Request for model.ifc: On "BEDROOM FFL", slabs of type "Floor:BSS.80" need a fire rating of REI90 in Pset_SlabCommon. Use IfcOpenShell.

First a look at what the model holds.

```python
import ifcopenshell
import ifcopenshell.util.element

model = ifcopenshell.open("model.ifc")
print(model.schema)
storey = next(s for s in model.by_type("IfcBuildingStorey") if s.Name == "BEDROOM FFL")
slabs = [e for e in ifcopenshell.util.element.get_decomposition(storey) if e.is_a("IfcSlab")]
seen = {}
for e in slabs:
    element_type = ifcopenshell.util.element.get_type(e)
    key = (element_type.Name if element_type != e and element_type else None, ifcopenshell.util.element.get_pset(e, "Pset_SlabCommon", "FireRating"))
    seen[key] = seen.get(key, 0) + 1
for (name, value), count in sorted(seen.items(), key=str):
    print(count, "x", name, "|", value)
```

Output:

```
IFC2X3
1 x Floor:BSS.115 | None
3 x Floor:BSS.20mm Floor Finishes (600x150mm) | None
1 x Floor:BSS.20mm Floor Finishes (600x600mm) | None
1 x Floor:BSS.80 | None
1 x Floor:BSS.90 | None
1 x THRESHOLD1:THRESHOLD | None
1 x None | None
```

```python
import ifcopenshell
import ifcopenshell.api.pset
import ifcopenshell.util.element

model = ifcopenshell.open("model.ifc")

storey = next(s for s in model.by_type("IfcBuildingStorey") if s.Name == "BEDROOM FFL")
slabs = [e for e in ifcopenshell.util.element.get_decomposition(storey) if e.is_a("IfcSlab")]

count = 0
for e in slabs:
    element_type = ifcopenshell.util.element.get_type(e)
    if element_type in (None, e) or element_type.Name != "Floor:BSS.80":
        continue
    # add_pset returns the element's existing set when there is one.
    pset = ifcopenshell.api.pset.add_pset(model, product=e, name="Pset_SlabCommon")
    ifcopenshell.api.pset.edit_pset(model, pset=pset, properties={"FireRating": "REI90"})
    count += 1

print(count, "slabs updated")

model.write("model_updated.ifc")
```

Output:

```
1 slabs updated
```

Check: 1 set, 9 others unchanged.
